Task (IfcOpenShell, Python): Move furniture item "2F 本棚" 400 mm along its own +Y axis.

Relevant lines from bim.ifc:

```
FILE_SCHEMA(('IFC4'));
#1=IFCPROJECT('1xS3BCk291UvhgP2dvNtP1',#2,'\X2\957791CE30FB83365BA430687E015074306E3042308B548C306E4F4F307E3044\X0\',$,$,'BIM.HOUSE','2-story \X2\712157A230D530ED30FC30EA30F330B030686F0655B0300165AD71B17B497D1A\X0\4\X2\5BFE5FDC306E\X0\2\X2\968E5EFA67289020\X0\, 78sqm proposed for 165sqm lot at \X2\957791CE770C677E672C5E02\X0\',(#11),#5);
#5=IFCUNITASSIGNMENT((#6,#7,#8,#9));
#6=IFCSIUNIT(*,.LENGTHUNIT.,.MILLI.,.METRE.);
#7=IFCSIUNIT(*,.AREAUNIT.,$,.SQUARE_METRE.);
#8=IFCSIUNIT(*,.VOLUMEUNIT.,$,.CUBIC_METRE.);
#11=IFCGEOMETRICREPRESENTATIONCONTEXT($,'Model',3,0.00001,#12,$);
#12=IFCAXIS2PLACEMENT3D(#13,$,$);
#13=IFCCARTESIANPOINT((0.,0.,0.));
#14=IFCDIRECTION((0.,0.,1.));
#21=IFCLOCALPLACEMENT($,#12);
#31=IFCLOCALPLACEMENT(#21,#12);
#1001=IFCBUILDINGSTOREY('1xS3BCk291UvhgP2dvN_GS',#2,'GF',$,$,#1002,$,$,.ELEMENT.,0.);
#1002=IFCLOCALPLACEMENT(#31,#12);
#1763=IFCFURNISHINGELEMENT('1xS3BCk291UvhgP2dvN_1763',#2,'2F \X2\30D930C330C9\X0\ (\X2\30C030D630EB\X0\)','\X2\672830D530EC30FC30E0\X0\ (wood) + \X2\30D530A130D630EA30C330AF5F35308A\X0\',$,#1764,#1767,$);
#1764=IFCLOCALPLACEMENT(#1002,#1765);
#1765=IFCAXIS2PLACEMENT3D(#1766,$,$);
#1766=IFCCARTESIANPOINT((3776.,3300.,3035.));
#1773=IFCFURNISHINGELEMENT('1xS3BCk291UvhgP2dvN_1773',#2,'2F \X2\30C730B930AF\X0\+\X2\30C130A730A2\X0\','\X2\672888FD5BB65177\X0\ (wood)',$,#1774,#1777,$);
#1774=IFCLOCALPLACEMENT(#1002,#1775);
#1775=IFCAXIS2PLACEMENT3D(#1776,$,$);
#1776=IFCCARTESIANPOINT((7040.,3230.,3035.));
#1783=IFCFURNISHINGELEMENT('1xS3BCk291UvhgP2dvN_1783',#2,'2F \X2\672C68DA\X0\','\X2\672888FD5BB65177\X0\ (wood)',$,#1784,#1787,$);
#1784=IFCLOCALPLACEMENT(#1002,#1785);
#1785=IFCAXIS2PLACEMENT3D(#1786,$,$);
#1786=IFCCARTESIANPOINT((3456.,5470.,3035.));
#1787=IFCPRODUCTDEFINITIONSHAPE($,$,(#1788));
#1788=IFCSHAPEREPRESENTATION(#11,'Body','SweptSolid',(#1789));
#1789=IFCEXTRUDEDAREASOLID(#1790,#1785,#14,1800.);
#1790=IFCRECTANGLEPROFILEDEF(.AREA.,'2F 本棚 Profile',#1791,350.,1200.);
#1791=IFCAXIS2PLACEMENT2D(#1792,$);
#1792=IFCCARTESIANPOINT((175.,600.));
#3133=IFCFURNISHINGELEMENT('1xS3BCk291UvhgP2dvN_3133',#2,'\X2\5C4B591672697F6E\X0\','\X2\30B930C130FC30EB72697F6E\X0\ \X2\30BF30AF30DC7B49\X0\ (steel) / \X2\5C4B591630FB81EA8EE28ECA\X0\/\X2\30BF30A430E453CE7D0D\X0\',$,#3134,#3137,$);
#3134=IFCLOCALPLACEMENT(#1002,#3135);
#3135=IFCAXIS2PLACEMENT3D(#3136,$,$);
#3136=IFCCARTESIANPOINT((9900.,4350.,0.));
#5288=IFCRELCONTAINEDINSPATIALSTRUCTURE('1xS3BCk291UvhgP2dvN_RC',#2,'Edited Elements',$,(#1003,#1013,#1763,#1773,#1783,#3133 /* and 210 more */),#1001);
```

```python
import ifcopenshell
import ifcopenshell.api.geometry
import ifcopenshell.util.placement
import ifcopenshell.util.unit

model = ifcopenshell.open("bim.ifc")
unit_scale = ifcopenshell.util.unit.calculate_unit_scale(model)

item = model.by_guid("1xS3BCk291UvhgP2dvN_1783")
matrix = ifcopenshell.util.placement.get_local_placement(item.ObjectPlacement)
matrix[:3, 3] += matrix[:3, 1] * 0.4 / unit_scale
ifcopenshell.api.geometry.edit_object_placement(model, product=item, matrix=matrix, is_si=False)

print(ifcopenshell.util.placement.get_local_placement(item.ObjectPlacement).round(3) + 0.0)

model.write("bim_rev.ifc")
```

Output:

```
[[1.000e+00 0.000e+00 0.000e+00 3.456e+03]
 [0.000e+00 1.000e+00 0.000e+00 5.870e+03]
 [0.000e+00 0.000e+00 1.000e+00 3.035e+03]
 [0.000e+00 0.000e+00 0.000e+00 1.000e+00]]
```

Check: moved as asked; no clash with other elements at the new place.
